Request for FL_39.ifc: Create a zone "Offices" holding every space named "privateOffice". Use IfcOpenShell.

First a look at what the model holds.

```python
import ifcopenshell

model = ifcopenshell.open("FL_39.ifc")
print(model.schema)
seen = {}
for space in model.by_type("IfcSpace"):
    seen[space.LongName] = seen.get(space.LongName, 0) + 1
for name, count in sorted(seen.items(), key=str):
    print(count, "x", name)
print("zones:", [z.Name for z in model.by_type("IfcZone")][:20])
```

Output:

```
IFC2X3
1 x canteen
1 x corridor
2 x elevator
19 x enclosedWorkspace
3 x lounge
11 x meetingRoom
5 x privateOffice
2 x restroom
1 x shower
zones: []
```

```python
import ifcopenshell
import ifcopenshell.api.group
import ifcopenshell.api.root

model = ifcopenshell.open("FL_39.ifc")

names = {"privateOffice"}
spaces = [s for s in model.by_type("IfcSpace") if s.LongName in names]

zone = ifcopenshell.api.root.create_entity(model, ifc_class="IfcZone", name="Offices")
ifcopenshell.api.group.assign_group(model, products=spaces, group=zone)
print(len(spaces), "spaces in", zone.Name)

model.write("FL_39_updated.ifc")
```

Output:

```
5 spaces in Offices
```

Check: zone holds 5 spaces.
